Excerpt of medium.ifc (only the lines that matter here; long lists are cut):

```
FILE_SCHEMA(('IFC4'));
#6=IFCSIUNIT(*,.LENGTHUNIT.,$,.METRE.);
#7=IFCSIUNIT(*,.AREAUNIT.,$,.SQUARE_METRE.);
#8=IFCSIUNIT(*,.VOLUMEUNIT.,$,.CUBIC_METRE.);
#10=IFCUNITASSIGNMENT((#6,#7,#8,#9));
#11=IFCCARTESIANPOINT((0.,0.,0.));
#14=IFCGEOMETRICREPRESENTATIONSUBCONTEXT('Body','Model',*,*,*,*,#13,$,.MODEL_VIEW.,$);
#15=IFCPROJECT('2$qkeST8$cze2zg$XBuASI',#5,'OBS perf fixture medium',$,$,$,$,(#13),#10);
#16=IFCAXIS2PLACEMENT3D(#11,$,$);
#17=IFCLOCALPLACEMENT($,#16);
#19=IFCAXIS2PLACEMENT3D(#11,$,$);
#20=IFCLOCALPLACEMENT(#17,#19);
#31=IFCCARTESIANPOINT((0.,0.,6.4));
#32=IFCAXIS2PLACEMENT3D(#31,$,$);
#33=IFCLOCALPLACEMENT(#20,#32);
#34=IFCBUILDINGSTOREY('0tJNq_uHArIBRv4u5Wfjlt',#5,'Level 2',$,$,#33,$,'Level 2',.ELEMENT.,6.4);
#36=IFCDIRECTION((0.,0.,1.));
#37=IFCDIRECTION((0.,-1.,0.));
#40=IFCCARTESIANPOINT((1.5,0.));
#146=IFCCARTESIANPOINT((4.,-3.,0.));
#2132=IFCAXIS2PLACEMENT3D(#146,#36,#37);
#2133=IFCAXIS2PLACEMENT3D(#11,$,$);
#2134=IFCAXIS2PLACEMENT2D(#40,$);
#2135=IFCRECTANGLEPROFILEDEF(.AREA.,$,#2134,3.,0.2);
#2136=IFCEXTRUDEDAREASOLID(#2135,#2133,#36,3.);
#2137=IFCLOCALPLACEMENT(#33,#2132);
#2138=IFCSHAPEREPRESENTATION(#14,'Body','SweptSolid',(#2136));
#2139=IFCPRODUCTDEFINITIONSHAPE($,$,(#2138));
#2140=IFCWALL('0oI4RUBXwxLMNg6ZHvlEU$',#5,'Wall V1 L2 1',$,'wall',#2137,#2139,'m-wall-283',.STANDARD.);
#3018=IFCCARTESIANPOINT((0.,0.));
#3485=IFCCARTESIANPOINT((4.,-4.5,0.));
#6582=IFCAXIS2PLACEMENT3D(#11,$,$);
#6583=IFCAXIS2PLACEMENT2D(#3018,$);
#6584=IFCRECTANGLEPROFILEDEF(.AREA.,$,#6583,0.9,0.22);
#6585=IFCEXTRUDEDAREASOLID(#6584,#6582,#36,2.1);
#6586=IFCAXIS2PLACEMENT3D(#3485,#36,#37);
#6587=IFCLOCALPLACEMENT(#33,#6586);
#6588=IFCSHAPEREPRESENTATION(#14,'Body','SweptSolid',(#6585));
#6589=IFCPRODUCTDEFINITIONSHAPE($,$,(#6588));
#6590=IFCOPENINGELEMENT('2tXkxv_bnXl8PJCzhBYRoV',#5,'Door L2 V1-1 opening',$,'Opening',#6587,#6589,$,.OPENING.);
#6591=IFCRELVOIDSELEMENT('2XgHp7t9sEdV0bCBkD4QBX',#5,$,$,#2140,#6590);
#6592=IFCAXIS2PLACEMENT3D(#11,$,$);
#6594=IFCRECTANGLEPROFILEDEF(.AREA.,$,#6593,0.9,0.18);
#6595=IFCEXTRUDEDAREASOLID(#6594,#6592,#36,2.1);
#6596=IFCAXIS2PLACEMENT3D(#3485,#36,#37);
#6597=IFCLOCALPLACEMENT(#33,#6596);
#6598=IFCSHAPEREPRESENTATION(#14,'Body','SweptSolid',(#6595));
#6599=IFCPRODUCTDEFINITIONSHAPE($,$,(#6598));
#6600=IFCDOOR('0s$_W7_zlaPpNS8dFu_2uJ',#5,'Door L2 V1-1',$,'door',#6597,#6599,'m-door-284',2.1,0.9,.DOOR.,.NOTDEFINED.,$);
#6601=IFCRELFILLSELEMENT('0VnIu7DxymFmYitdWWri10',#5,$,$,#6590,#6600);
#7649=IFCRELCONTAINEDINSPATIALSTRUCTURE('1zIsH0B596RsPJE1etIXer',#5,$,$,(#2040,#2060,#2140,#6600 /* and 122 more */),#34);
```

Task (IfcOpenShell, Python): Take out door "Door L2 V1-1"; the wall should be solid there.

```python
import ifcopenshell
import ifcopenshell.api.feature
import ifcopenshell.api.root
import ifcopenshell.geom
import ifcopenshell.util.shape

model = ifcopenshell.open("medium.ifc")
settings = ifcopenshell.geom.settings()


def volume(element):
    """Net volume in cubic metres, openings subtracted."""
    shape = ifcopenshell.geom.create_shape(settings, element)
    return ifcopenshell.util.shape.get_volume(shape.geometry)


door = model.by_id(6600)
opening = door.FillsVoids[0].RelatingOpeningElement
wall = opening.VoidsElements[0].RelatingBuildingElement
before = volume(wall)

ifcopenshell.api.root.remove_product(model, product=door)
ifcopenshell.api.feature.remove_feature(model, feature=opening)

after = volume(wall)

print(f"wall volume {before:.3f} -> {after:.3f} m3")

model.write("medium_v2.ifc")
```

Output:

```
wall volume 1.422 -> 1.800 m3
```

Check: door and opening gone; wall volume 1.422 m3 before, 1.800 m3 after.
